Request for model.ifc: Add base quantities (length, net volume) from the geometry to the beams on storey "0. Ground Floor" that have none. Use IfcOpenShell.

First a look at what the model holds.

```python
import ifcopenshell
import ifcopenshell.util.element
import ifcopenshell.util.unit

model = ifcopenshell.open("model.ifc")
print(model.schema)
for unit_type in ("LENGTHUNIT", "AREAUNIT", "VOLUMEUNIT"):
    print(unit_type, ifcopenshell.util.unit.calculate_unit_scale(model, unit_type))
storey = next(s for s in model.by_type("IfcBuildingStorey") if s.Name == "0. Ground Floor")
beams = [e for e in ifcopenshell.util.element.get_decomposition(storey) if e.is_a("IfcBeam")]
for e in sorted(beams, key=lambda e: e.id()):
    print(e.id(), e.is_a(), e.Name, list(ifcopenshell.util.element.get_psets(e, qtos_only=True)), sep=" | ")
```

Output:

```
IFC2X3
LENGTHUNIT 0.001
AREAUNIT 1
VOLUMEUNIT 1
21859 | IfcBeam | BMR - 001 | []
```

```python
import ifcopenshell
import ifcopenshell.api.pset
import ifcopenshell.geom
import ifcopenshell.util.element
import ifcopenshell.util.shape
import ifcopenshell.util.unit

model = ifcopenshell.open("model.ifc")
unit_scale = ifcopenshell.util.unit.calculate_unit_scale(model)
volume_scale = ifcopenshell.util.unit.calculate_unit_scale(model, "VOLUMEUNIT")
settings = ifcopenshell.geom.settings()

storey = next(s for s in model.by_type("IfcBuildingStorey") if s.Name == "0. Ground Floor")
beams = [e for e in ifcopenshell.util.element.get_decomposition(storey) if e.is_a("IfcBeam")]

for e in sorted(beams, key=lambda e: e.id()):
    if ifcopenshell.util.element.get_psets(e, qtos_only=True, should_inherit=False):
        continue
    # Geometry comes back in metres, in the element's own axes.
    shape = ifcopenshell.geom.create_shape(settings, e)
    values = {
        "Length": ifcopenshell.util.shape.get_max_xyz(shape.geometry) / unit_scale,
        "NetVolume": ifcopenshell.util.shape.get_volume(shape.geometry) / volume_scale,
    }
    qto = ifcopenshell.api.pset.add_qto(model, product=e, name="BaseQuantities")
    ifcopenshell.api.pset.edit_qto(model, qto=qto, properties=values)
    print(e.id(), {k: round(v, 3) for k, v in values.items()})

model.write("model_rev.ifc")
```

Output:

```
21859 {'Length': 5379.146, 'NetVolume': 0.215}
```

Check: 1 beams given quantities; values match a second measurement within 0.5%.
